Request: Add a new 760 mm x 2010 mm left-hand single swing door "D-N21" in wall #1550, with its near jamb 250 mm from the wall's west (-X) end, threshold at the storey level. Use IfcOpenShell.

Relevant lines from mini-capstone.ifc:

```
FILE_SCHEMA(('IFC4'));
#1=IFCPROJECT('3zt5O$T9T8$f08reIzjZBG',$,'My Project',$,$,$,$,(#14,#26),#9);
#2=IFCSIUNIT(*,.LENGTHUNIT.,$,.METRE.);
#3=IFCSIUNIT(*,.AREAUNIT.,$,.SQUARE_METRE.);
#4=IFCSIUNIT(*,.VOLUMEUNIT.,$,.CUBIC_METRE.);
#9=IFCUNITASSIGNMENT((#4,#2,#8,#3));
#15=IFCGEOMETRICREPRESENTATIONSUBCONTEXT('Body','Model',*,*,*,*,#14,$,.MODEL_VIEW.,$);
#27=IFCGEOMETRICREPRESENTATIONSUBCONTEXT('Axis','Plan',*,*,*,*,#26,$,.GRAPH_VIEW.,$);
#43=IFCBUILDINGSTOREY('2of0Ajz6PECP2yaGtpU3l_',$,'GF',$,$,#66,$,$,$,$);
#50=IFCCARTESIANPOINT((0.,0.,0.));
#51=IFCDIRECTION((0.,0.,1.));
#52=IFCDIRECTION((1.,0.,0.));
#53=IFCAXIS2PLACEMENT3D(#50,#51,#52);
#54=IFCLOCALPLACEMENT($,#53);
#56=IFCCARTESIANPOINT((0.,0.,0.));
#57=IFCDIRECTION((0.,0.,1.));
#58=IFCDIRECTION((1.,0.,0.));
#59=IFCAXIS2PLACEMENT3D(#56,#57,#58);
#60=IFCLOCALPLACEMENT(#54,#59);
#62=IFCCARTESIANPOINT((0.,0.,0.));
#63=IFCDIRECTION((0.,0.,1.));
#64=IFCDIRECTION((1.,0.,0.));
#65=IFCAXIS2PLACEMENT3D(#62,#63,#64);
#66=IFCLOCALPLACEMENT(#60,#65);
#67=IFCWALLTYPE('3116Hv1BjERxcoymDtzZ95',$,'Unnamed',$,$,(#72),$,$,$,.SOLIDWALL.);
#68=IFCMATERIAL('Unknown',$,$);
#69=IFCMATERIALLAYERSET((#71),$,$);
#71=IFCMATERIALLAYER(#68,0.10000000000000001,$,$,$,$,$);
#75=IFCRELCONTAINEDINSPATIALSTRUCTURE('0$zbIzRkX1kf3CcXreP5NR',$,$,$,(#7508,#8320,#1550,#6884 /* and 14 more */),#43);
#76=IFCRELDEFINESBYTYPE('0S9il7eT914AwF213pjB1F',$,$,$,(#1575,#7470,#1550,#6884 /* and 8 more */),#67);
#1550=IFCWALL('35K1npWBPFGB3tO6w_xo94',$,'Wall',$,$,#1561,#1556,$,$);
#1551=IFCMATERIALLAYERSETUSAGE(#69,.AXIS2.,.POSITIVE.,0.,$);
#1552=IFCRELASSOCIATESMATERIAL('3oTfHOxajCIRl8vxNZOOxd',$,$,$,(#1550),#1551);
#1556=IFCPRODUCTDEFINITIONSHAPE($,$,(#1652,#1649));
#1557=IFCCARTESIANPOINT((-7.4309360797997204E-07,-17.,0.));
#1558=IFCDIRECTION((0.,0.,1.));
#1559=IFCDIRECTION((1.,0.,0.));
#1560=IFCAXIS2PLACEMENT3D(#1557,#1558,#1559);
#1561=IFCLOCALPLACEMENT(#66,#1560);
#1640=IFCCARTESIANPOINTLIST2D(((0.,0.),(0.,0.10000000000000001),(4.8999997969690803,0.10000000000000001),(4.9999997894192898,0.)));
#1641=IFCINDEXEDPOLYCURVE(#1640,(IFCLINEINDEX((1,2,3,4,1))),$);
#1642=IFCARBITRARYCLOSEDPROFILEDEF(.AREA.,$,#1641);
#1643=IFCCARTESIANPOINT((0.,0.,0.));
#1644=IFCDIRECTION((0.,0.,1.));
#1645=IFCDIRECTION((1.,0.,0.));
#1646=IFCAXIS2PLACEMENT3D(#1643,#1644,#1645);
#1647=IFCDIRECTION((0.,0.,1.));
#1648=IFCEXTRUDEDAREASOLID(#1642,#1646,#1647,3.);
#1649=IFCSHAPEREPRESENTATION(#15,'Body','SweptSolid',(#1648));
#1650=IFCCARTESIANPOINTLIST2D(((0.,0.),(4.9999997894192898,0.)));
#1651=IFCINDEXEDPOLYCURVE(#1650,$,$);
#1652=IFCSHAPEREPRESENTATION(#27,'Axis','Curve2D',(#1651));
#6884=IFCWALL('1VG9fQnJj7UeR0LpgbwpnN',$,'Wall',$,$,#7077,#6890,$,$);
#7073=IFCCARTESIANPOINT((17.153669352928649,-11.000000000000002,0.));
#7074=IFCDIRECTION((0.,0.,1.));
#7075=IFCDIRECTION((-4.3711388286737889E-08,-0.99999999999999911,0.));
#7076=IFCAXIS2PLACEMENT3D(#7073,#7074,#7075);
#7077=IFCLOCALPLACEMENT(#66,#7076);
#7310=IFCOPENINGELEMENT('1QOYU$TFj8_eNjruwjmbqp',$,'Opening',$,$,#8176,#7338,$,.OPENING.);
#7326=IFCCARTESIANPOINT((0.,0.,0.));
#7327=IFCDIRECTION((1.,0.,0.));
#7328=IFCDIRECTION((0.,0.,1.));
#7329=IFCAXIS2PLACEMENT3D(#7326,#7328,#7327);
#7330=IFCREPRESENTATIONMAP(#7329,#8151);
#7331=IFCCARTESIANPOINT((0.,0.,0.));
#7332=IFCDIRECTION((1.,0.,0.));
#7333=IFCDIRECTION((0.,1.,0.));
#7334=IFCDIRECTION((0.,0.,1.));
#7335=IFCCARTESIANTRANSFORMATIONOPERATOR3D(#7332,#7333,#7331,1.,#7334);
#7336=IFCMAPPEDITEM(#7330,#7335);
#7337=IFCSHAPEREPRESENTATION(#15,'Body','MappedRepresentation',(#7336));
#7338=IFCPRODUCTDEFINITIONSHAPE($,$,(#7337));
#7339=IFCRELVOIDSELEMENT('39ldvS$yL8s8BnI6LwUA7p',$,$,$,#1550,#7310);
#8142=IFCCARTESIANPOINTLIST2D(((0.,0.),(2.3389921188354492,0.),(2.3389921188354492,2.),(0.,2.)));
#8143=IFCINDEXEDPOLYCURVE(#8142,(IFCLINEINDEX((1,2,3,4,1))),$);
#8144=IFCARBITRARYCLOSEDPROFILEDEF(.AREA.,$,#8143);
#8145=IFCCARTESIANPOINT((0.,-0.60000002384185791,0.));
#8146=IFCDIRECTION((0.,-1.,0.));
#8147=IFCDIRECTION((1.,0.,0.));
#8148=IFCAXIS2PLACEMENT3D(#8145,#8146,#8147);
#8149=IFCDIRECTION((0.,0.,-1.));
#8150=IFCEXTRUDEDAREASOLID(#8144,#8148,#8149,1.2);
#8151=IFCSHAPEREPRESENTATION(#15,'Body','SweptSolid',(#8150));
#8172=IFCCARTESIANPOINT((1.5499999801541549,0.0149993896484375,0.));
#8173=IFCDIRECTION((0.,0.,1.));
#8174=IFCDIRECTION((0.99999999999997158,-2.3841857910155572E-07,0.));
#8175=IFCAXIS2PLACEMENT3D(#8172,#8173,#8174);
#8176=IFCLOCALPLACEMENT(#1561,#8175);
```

```python
import numpy as np
import ifcopenshell
import ifcopenshell.api.feature
import ifcopenshell.api.geometry
import ifcopenshell.api.root
import ifcopenshell.api.spatial
import ifcopenshell.geom
import ifcopenshell.util.element
import ifcopenshell.util.placement
import ifcopenshell.util.representation
import ifcopenshell.util.shape
import ifcopenshell.util.unit

model = ifcopenshell.open("mini-capstone.ifc")
unit_scale = ifcopenshell.util.unit.calculate_unit_scale(model)
settings = ifcopenshell.geom.settings()


def volume(element):
    """Net volume in cubic metres, openings subtracted."""
    shape = ifcopenshell.geom.create_shape(settings, element)
    return ifcopenshell.util.shape.get_volume(shape.geometry)


wall = model.by_guid("35K1npWBPFGB3tO6w_xo94")
storey = ifcopenshell.util.element.get_container(wall, ifc_class="IfcBuildingStorey")
context = ifcopenshell.util.representation.get_context(model, "Model", "Body", "MODEL_VIEW")
before = volume(wall)

width, height, from_end, sill = 0.76, 2.01, 0.25, 0.0  # metres

# The wall runs along its own X axis, and the end named is its -X end.
wall_shape = ifcopenshell.geom.create_shape(settings, wall)
x, y, z = ifcopenshell.util.shape.get_vertices(wall_shape.geometry).T
start = x.min() + from_end
face, thickness = float(y.min()), float(y.max() - y.min())
wall_matrix = ifcopenshell.util.placement.get_local_placement(wall.ObjectPlacement)
level = ifcopenshell.util.placement.get_local_placement(storey.ObjectPlacement)[2, 3]


def in_wall(x, y):
    """Placement at x, y metres in the wall's axes, at sill height."""
    matrix = wall_matrix.copy()
    matrix[:, 3] = wall_matrix @ np.array([x / unit_scale, y / unit_scale, 0.0, 1.0])
    matrix[2, 3] = level + sill / unit_scale
    return matrix


# Opening: a box that overshoots both wall faces by 50 mm.
opening = ifcopenshell.api.root.create_entity(model, ifc_class="IfcOpeningElement", predefined_type="OPENING")
box = ifcopenshell.api.geometry.add_wall_representation(
    model, context=context, length=width, height=height, thickness=thickness + 0.1
)
ifcopenshell.api.geometry.assign_representation(model, product=opening, representation=box)
ifcopenshell.api.geometry.edit_object_placement(model, product=opening, matrix=in_wall(start, face - 0.05), is_si=False)
ifcopenshell.api.feature.add_feature(model, feature=opening, element=wall)

door = ifcopenshell.api.root.create_entity(model, ifc_class="IfcDoor", name="D-N21", predefined_type="DOOR")
door.OverallWidth, door.OverallHeight = width / unit_scale, height / unit_scale
door.OperationType = "SINGLE_SWING_LEFT"
body = ifcopenshell.api.geometry.add_door_representation(
    model,
    context=context,
    overall_width=door.OverallWidth,
    overall_height=door.OverallHeight,
    operation_type="SINGLE_SWING_LEFT",
    lining_properties={"LiningDepth": thickness / unit_scale, "ThresholdDepth": thickness / unit_scale},
)
ifcopenshell.api.geometry.assign_representation(model, product=door, representation=body)
ifcopenshell.api.spatial.assign_container(model, products=[door], relating_structure=storey)
ifcopenshell.api.feature.add_filling(model, opening=opening, element=door)

# The lining spans the wall, so the door starts at the wall face.
ifcopenshell.api.geometry.edit_object_placement(model, product=door, matrix=in_wall(start, face), is_si=False)

after = volume(wall)

print(f"wall volume {before:.3f} -> {after:.3f} m3")

model.write("mini-capstone_rev.ifc")
```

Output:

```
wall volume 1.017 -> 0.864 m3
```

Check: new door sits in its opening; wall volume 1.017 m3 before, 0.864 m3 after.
